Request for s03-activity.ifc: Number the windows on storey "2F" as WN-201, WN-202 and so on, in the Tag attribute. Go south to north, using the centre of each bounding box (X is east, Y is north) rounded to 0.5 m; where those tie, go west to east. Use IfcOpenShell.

First a look at what the model holds.

```python
import ifcopenshell
import ifcopenshell.util.element
import ifcopenshell.util.placement

model = ifcopenshell.open("s03-activity.ifc")
print(model.schema)
storey = next(s for s in model.by_type("IfcBuildingStorey") if s.Name == "2F")
windows = [e for e in ifcopenshell.util.element.get_decomposition(storey) if e.is_a("IfcWindow")]
for e in sorted(windows, key=lambda e: e.id()):
    origin = ifcopenshell.util.placement.get_local_placement(e.ObjectPlacement)[:3, 3]
    print(e.id(), e.Tag, e.Name, origin.round(2) + 0.0, sep=" | ")
```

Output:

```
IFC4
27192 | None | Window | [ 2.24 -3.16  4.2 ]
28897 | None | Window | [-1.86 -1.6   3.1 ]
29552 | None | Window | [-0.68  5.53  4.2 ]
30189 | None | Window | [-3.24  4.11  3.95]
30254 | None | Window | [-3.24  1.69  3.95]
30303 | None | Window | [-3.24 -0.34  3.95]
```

```python
import ifcopenshell
import ifcopenshell.geom
import ifcopenshell.util.element
import ifcopenshell.util.shape

model = ifcopenshell.open("s03-activity.ifc")
settings = ifcopenshell.geom.settings()
settings.set("use-world-coords", True)


def centre(element):
    shape = ifcopenshell.geom.create_shape(settings, element)
    return ifcopenshell.util.shape.get_bbox_centroid(shape.geometry)


storey = next(s for s in model.by_type("IfcBuildingStorey") if s.Name == "2F")
windows = [e for e in ifcopenshell.util.element.get_decomposition(storey) if e.is_a("IfcWindow")]

# Insertion points can sit at a corner or the storey origin, so sort by the geometry (in metres).
centres = {e: centre(e) for e in windows}
windows.sort(key=lambda e: (round(centres[e][1] / 0.5), centres[e][0]))

for i, e in enumerate(windows, start=1):
    number = f"WN-2{i:02d}"
    e.Tag = number
    print(e.id(), number)

model.write("s03-activity-out.ifc")
```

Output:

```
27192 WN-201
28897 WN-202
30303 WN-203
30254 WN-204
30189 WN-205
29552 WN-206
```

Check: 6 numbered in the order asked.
